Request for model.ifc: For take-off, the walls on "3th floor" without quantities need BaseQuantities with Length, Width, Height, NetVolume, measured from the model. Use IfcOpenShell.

First a look at what the model holds.

```python
import ifcopenshell
import ifcopenshell.util.element
import ifcopenshell.util.unit

model = ifcopenshell.open("model.ifc")
print(model.schema)
for unit_type in ("LENGTHUNIT", "AREAUNIT", "VOLUMEUNIT"):
    print(unit_type, ifcopenshell.util.unit.calculate_unit_scale(model, unit_type))
storey = next(s for s in model.by_type("IfcBuildingStorey") if s.Name == "3th floor")
walls = [e for e in ifcopenshell.util.element.get_decomposition(storey) if e.is_a("IfcWall")]
for e in sorted(walls, key=lambda e: e.id()):
    print(e.id(), e.is_a(), e.Name, list(ifcopenshell.util.element.get_psets(e, qtos_only=True)), sep=" | ")
```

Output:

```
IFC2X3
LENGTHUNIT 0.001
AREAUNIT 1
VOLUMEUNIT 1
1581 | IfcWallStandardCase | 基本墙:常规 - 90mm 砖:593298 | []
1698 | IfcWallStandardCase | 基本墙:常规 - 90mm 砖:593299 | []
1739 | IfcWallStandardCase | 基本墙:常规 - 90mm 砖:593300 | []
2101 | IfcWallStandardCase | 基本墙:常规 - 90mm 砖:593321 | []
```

```python
import ifcopenshell
import ifcopenshell.api.pset
import ifcopenshell.geom
import ifcopenshell.util.element
import ifcopenshell.util.shape
import ifcopenshell.util.unit

model = ifcopenshell.open("model.ifc")
unit_scale = ifcopenshell.util.unit.calculate_unit_scale(model)
volume_scale = ifcopenshell.util.unit.calculate_unit_scale(model, "VOLUMEUNIT")
settings = ifcopenshell.geom.settings()

storey = next(s for s in model.by_type("IfcBuildingStorey") if s.Name == "3th floor")
walls = [e for e in ifcopenshell.util.element.get_decomposition(storey) if e.is_a("IfcWall")]

for e in sorted(walls, key=lambda e: e.id()):
    if ifcopenshell.util.element.get_psets(e, qtos_only=True, should_inherit=False):
        continue
    # Geometry comes back in metres, in the element's own axes.
    shape = ifcopenshell.geom.create_shape(settings, e)
    values = {
        "Length": ifcopenshell.util.shape.get_x(shape.geometry) / unit_scale,
        "Width": ifcopenshell.util.shape.get_y(shape.geometry) / unit_scale,
        "Height": ifcopenshell.util.shape.get_z(shape.geometry) / unit_scale,
        "NetVolume": ifcopenshell.util.shape.get_volume(shape.geometry) / volume_scale,
    }
    qto = ifcopenshell.api.pset.add_qto(model, product=e, name="BaseQuantities")
    ifcopenshell.api.pset.edit_qto(model, qto=qto, properties=values)
    print(e.id(), {k: round(v, 3) for k, v in values.items()})

model.write("model_v2.ifc")
```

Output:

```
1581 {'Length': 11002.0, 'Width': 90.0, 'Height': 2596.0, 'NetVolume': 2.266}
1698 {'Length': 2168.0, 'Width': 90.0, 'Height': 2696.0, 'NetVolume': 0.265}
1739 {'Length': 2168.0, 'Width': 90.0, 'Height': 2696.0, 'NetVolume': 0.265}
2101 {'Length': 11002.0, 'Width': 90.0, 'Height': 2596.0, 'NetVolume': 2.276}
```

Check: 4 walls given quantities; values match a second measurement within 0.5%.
